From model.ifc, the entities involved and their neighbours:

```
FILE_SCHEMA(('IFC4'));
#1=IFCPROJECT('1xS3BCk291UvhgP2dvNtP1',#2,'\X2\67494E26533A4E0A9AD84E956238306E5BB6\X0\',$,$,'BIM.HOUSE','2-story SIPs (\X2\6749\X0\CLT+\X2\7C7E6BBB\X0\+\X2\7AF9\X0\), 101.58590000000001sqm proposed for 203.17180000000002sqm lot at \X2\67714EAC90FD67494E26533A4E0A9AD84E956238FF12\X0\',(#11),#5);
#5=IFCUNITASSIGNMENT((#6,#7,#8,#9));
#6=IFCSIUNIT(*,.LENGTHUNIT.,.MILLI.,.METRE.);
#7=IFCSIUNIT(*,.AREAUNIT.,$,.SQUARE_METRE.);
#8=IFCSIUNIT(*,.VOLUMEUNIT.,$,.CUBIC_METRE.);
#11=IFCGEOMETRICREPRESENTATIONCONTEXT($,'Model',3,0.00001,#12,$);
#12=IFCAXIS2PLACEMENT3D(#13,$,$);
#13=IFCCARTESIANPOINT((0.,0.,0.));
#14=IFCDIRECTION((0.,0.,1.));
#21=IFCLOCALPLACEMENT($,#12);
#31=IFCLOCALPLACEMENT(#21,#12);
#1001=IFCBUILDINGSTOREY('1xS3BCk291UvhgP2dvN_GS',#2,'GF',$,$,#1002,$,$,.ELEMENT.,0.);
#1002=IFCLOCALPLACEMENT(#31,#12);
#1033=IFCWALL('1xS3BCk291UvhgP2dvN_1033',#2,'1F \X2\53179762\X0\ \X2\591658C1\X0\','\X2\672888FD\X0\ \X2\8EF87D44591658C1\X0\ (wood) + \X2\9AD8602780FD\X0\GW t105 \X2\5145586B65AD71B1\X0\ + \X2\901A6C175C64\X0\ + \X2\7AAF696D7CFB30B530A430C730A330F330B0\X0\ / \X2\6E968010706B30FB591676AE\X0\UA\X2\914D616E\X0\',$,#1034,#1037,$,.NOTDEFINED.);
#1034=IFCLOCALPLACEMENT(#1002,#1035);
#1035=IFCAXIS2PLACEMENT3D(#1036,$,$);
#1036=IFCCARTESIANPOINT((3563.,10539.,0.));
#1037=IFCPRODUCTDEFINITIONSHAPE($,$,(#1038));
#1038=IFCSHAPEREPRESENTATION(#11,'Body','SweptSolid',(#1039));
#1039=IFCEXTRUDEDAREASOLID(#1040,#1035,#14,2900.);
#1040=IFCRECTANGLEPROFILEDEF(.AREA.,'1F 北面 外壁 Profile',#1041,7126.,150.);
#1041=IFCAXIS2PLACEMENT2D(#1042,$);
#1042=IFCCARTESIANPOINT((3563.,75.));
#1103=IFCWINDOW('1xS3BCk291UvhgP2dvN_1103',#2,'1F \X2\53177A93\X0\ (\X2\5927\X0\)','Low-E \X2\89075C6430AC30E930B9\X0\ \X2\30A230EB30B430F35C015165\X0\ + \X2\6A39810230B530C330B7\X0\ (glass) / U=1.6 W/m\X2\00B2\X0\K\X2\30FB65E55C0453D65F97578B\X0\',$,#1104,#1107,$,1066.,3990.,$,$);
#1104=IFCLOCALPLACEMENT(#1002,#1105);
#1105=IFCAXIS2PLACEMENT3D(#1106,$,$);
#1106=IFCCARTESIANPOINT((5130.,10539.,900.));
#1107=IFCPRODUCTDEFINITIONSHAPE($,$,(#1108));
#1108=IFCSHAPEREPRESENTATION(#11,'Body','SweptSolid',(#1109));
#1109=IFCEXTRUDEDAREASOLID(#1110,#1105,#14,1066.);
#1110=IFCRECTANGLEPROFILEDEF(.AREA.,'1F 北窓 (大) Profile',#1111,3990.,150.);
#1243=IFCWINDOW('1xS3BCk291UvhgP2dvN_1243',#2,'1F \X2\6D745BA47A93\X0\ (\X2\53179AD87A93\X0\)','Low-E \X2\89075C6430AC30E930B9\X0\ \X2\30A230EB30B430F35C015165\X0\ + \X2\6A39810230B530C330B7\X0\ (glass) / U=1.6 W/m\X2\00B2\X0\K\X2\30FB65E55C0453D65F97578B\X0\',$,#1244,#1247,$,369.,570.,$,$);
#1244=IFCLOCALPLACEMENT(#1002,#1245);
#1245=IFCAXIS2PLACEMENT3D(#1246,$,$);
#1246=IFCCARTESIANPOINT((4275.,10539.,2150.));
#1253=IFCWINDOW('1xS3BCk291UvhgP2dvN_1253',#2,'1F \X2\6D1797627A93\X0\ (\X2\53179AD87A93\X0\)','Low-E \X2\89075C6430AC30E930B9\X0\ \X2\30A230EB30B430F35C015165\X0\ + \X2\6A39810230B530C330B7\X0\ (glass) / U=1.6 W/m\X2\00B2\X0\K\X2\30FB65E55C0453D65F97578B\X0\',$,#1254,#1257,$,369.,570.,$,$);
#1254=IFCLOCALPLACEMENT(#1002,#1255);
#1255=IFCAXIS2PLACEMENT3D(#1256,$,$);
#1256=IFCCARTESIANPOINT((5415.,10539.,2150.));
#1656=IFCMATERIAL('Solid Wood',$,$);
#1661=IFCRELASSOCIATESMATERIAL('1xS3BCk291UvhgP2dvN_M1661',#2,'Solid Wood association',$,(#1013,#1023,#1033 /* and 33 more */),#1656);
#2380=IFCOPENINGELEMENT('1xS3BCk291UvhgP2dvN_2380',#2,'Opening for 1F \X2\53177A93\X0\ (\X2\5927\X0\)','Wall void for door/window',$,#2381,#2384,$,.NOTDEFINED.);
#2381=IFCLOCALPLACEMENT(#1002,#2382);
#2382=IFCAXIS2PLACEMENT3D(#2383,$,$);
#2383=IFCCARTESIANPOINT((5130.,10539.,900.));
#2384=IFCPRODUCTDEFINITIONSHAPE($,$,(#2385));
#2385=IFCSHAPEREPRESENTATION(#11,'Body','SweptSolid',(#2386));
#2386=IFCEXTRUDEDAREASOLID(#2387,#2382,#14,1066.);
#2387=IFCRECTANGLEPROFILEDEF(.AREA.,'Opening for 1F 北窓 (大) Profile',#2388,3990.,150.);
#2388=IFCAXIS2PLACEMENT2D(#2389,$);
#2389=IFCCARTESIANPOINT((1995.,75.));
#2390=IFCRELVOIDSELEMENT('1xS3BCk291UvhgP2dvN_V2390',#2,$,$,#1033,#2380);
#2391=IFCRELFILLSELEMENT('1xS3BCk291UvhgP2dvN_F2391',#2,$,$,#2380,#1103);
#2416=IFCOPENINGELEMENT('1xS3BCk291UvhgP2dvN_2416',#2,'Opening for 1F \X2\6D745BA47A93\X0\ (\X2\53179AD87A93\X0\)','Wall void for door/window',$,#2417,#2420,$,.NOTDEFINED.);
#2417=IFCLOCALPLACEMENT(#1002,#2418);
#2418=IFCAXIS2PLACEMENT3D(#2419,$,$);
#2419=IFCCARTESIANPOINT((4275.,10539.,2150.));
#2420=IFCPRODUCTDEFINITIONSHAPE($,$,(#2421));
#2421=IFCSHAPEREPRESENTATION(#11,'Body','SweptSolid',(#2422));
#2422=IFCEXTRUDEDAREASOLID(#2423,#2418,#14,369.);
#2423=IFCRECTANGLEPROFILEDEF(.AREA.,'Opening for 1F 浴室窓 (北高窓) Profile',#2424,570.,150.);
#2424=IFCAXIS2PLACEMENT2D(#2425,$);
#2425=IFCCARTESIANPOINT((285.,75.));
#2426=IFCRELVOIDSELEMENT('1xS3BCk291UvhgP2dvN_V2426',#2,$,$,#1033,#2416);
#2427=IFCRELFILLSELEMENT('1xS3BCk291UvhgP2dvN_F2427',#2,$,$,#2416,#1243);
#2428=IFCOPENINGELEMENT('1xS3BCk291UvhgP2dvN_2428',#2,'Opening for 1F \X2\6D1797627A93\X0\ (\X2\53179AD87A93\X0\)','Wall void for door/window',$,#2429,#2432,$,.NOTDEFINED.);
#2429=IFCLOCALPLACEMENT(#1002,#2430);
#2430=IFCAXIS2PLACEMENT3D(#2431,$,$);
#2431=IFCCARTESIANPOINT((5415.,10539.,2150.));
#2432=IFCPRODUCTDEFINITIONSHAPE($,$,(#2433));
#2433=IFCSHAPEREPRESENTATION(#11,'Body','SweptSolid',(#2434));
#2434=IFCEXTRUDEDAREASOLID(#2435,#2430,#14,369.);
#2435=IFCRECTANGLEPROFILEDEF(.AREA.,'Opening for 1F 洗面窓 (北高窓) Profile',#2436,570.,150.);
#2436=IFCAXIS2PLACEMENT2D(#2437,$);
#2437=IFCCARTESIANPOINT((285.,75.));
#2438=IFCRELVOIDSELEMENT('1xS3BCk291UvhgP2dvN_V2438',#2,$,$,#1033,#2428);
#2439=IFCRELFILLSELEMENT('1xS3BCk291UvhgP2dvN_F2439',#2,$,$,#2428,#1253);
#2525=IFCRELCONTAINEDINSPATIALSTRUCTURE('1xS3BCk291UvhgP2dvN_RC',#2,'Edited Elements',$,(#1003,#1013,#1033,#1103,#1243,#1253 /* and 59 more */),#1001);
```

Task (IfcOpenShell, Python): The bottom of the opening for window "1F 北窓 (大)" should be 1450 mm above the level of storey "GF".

```python
import numpy as np
import ifcopenshell
import ifcopenshell.api.geometry
import ifcopenshell.geom
import ifcopenshell.util.element
import ifcopenshell.util.placement
import ifcopenshell.util.shape
import ifcopenshell.util.unit

model = ifcopenshell.open("model.ifc")
unit_scale = ifcopenshell.util.unit.calculate_unit_scale(model)

window = model.by_guid("1xS3BCk291UvhgP2dvN_1103")
opening = window.FillsVoids[0].RelatingOpeningElement
storey = ifcopenshell.util.element.get_container(window, ifc_class="IfcBuildingStorey")
level = ifcopenshell.util.placement.get_local_placement(storey.ObjectPlacement)[2, 3]

# The opening's origin need not be at the sill, so measure its lowest point.
shape = ifcopenshell.geom.create_shape(ifcopenshell.geom.settings(), opening)
bottom = ifcopenshell.util.shape.get_shape_bottom_elevation(shape, shape.geometry) / unit_scale
dz = level + 1450.0 - bottom

shift = np.array([0.0, 0.0, dz])
# The window is not placed relative to its opening, so move both.
for product in (opening, window):
    matrix = ifcopenshell.util.placement.get_local_placement(product.ObjectPlacement)
    matrix[:3, 3] += shift
    ifcopenshell.api.geometry.edit_object_placement(model, product=product, matrix=matrix, is_si=False)

print(f"moved by {dz * unit_scale:+.3f} m")

model.write("model_updated.ifc")
```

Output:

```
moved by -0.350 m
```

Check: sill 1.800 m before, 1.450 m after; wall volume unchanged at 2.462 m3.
